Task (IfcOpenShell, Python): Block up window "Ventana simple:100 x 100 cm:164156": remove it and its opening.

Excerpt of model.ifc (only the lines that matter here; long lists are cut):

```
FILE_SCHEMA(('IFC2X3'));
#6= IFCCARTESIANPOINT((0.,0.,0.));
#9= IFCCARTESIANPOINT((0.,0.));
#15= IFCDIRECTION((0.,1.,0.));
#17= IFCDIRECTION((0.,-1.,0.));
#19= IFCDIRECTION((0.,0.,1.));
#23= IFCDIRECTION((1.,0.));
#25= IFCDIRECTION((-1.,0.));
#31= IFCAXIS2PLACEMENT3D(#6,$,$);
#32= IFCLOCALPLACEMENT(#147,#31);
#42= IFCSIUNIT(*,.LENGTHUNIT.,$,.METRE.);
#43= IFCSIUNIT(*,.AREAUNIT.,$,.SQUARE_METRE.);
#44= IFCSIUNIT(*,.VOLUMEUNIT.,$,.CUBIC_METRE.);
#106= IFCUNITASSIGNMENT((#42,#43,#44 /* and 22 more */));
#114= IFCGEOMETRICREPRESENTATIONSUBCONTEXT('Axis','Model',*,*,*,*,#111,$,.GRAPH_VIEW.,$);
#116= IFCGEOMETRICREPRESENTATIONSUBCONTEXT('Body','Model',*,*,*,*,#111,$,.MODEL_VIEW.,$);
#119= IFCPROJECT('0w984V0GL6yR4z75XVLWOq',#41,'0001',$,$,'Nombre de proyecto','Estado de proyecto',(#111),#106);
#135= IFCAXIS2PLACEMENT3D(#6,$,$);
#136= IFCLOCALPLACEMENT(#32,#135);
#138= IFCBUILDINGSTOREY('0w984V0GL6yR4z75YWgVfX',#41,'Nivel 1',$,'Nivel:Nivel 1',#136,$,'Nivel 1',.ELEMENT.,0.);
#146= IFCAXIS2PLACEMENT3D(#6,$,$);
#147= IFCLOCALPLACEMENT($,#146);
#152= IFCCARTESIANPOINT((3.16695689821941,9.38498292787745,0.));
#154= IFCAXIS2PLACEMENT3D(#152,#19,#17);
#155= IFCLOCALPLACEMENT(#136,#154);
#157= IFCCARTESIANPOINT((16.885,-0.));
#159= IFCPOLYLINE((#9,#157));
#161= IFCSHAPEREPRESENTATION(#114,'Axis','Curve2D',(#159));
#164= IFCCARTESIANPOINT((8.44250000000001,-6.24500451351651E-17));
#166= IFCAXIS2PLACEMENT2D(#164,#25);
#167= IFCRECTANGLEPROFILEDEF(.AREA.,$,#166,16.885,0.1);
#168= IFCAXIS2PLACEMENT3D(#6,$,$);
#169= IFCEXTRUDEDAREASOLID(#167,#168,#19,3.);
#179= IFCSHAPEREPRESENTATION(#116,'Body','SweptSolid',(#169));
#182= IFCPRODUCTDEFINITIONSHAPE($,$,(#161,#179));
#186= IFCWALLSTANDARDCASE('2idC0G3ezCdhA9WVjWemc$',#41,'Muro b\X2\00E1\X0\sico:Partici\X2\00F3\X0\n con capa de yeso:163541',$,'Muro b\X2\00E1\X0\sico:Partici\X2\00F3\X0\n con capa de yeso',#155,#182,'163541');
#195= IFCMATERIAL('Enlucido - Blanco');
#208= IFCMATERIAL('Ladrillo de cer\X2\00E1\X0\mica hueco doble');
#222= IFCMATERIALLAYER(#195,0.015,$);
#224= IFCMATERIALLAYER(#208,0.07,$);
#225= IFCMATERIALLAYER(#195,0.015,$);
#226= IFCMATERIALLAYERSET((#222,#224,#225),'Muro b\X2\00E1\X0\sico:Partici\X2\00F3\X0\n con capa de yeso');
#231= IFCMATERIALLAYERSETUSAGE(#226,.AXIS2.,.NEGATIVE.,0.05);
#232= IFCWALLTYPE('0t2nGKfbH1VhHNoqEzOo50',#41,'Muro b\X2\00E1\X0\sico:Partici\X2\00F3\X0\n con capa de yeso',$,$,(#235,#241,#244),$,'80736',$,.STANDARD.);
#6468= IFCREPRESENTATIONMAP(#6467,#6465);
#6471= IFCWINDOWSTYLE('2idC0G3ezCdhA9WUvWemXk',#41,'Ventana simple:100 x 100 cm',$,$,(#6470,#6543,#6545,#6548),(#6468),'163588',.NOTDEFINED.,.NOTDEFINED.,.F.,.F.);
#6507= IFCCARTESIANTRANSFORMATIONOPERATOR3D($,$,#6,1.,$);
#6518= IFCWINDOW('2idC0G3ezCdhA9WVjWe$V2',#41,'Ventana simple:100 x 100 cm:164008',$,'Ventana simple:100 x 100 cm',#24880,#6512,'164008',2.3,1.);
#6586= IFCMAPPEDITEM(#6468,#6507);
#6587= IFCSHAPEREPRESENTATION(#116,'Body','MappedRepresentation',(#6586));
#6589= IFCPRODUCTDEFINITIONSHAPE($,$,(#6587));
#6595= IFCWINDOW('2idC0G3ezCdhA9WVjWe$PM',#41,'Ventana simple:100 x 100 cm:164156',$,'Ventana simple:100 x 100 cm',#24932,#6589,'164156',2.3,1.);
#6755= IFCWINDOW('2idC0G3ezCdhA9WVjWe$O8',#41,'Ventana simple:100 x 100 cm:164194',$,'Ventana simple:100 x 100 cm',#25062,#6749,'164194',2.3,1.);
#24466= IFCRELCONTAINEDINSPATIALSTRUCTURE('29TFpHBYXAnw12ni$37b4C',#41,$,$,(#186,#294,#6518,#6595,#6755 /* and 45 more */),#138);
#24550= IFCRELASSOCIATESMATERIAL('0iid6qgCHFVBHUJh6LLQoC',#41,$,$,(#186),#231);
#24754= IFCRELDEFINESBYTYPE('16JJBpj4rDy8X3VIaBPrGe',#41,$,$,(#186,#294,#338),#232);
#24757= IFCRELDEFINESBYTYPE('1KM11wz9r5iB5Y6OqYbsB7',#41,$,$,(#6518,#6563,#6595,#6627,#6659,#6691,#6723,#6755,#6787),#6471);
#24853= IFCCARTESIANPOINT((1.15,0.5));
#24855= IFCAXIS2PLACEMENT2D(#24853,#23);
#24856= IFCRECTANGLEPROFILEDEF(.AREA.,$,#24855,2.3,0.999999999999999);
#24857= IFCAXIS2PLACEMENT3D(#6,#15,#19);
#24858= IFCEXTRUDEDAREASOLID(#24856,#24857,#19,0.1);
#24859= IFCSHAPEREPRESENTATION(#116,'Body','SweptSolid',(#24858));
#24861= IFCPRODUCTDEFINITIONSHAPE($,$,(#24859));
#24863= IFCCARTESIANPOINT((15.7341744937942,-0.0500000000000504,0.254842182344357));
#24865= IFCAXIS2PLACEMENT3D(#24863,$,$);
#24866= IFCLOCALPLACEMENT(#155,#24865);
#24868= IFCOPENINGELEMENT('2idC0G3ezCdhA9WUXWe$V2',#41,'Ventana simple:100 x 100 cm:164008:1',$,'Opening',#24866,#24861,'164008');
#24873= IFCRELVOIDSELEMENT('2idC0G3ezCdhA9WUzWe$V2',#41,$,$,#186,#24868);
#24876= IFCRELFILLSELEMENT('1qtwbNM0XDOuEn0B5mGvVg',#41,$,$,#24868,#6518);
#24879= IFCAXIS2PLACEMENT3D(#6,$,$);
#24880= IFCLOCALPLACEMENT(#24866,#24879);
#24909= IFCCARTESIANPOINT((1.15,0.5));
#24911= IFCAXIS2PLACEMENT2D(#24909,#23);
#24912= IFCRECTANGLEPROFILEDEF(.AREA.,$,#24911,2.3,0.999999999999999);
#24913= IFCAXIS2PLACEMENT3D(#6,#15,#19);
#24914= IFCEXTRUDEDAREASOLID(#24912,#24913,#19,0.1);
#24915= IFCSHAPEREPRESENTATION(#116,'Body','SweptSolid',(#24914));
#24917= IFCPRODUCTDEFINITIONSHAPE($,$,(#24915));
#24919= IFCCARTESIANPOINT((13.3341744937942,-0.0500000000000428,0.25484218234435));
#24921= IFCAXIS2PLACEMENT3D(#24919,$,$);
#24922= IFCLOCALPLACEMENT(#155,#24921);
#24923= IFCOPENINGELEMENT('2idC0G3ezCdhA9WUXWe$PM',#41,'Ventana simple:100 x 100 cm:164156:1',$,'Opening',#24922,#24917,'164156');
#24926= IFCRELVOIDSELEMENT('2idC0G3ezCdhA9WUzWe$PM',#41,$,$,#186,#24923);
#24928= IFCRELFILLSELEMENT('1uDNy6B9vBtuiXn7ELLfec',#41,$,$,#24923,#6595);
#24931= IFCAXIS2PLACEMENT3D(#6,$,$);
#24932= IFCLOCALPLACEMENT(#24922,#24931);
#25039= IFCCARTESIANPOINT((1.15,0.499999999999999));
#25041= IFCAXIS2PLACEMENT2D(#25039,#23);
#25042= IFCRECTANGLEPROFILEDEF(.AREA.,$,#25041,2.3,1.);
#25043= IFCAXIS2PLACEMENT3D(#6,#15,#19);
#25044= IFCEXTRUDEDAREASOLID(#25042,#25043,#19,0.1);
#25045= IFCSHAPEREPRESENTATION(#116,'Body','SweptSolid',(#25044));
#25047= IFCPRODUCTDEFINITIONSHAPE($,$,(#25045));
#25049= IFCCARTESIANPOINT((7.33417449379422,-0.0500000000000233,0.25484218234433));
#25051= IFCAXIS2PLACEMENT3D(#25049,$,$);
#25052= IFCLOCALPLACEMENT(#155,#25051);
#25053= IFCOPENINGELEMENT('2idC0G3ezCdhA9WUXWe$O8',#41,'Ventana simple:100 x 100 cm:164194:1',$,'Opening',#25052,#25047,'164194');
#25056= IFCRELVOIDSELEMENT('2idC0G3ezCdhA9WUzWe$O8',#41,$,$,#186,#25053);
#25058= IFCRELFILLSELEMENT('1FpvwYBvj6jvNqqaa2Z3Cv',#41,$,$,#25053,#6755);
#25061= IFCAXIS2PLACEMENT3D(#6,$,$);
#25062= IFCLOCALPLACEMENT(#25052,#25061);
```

```python
import ifcopenshell
import ifcopenshell.api.feature
import ifcopenshell.api.root
import ifcopenshell.geom
import ifcopenshell.util.shape

model = ifcopenshell.open("model.ifc")
settings = ifcopenshell.geom.settings()


def volume(element):
    """Net volume in cubic metres, openings subtracted."""
    shape = ifcopenshell.geom.create_shape(settings, element)
    return ifcopenshell.util.shape.get_volume(shape.geometry)


window = model.by_guid("2idC0G3ezCdhA9WVjWe$PM")
opening = window.FillsVoids[0].RelatingOpeningElement
wall = opening.VoidsElements[0].RelatingBuildingElement
before = volume(wall)

ifcopenshell.api.root.remove_product(model, product=window)
ifcopenshell.api.feature.remove_feature(model, feature=opening)

after = volume(wall)

print(f"wall volume {before:.3f} -> {after:.3f} m3")

model.write("model-out.ifc")
```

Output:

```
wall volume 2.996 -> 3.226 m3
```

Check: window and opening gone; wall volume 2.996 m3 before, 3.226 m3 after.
